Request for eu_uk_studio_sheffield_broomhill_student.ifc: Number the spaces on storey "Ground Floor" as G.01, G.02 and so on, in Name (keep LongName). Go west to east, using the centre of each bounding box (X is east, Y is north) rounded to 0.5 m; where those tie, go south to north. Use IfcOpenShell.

First a look at what the model holds.

```python
import ifcopenshell
import ifcopenshell.util.element
import ifcopenshell.util.placement

model = ifcopenshell.open("eu_uk_studio_sheffield_broomhill_student.ifc")
print(model.schema)
storey = next(s for s in model.by_type("IfcBuildingStorey") if s.Name == "Ground Floor")
spaces = [e for e in ifcopenshell.util.element.get_decomposition(storey) if e.is_a("IfcSpace")]
for e in sorted(spaces, key=lambda e: e.id()):
    origin = ifcopenshell.util.placement.get_local_placement(e.ObjectPlacement)[:3, 3]
    print(e.id(), e.Name, e.LongName, origin.round(2) + 0.0, sep=" | ")
```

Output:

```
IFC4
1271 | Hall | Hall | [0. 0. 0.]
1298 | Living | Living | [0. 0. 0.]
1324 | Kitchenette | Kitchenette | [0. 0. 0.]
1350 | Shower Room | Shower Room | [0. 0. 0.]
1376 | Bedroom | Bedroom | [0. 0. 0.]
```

```python
import ifcopenshell
import ifcopenshell.geom
import ifcopenshell.util.element
import ifcopenshell.util.shape

model = ifcopenshell.open("eu_uk_studio_sheffield_broomhill_student.ifc")
settings = ifcopenshell.geom.settings()
settings.set("use-world-coords", True)


def centre(element):
    shape = ifcopenshell.geom.create_shape(settings, element)
    return ifcopenshell.util.shape.get_bbox_centroid(shape.geometry)


storey = next(s for s in model.by_type("IfcBuildingStorey") if s.Name == "Ground Floor")
spaces = [e for e in ifcopenshell.util.element.get_decomposition(storey) if e.is_a("IfcSpace")]

# Insertion points can sit at a corner or the storey origin, so sort by the geometry (in metres).
centres = {e: centre(e) for e in spaces}
spaces.sort(key=lambda e: (round(centres[e][0] / 0.5), centres[e][1]))

for i, e in enumerate(spaces, start=1):
    number = f"G.{i:02d}"
    e.Name = number
    print(e.id(), number)

model.write("eu_uk_studio_sheffield_broomhill_student_rev.ifc")
```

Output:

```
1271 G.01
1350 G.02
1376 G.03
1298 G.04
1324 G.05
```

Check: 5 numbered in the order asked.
